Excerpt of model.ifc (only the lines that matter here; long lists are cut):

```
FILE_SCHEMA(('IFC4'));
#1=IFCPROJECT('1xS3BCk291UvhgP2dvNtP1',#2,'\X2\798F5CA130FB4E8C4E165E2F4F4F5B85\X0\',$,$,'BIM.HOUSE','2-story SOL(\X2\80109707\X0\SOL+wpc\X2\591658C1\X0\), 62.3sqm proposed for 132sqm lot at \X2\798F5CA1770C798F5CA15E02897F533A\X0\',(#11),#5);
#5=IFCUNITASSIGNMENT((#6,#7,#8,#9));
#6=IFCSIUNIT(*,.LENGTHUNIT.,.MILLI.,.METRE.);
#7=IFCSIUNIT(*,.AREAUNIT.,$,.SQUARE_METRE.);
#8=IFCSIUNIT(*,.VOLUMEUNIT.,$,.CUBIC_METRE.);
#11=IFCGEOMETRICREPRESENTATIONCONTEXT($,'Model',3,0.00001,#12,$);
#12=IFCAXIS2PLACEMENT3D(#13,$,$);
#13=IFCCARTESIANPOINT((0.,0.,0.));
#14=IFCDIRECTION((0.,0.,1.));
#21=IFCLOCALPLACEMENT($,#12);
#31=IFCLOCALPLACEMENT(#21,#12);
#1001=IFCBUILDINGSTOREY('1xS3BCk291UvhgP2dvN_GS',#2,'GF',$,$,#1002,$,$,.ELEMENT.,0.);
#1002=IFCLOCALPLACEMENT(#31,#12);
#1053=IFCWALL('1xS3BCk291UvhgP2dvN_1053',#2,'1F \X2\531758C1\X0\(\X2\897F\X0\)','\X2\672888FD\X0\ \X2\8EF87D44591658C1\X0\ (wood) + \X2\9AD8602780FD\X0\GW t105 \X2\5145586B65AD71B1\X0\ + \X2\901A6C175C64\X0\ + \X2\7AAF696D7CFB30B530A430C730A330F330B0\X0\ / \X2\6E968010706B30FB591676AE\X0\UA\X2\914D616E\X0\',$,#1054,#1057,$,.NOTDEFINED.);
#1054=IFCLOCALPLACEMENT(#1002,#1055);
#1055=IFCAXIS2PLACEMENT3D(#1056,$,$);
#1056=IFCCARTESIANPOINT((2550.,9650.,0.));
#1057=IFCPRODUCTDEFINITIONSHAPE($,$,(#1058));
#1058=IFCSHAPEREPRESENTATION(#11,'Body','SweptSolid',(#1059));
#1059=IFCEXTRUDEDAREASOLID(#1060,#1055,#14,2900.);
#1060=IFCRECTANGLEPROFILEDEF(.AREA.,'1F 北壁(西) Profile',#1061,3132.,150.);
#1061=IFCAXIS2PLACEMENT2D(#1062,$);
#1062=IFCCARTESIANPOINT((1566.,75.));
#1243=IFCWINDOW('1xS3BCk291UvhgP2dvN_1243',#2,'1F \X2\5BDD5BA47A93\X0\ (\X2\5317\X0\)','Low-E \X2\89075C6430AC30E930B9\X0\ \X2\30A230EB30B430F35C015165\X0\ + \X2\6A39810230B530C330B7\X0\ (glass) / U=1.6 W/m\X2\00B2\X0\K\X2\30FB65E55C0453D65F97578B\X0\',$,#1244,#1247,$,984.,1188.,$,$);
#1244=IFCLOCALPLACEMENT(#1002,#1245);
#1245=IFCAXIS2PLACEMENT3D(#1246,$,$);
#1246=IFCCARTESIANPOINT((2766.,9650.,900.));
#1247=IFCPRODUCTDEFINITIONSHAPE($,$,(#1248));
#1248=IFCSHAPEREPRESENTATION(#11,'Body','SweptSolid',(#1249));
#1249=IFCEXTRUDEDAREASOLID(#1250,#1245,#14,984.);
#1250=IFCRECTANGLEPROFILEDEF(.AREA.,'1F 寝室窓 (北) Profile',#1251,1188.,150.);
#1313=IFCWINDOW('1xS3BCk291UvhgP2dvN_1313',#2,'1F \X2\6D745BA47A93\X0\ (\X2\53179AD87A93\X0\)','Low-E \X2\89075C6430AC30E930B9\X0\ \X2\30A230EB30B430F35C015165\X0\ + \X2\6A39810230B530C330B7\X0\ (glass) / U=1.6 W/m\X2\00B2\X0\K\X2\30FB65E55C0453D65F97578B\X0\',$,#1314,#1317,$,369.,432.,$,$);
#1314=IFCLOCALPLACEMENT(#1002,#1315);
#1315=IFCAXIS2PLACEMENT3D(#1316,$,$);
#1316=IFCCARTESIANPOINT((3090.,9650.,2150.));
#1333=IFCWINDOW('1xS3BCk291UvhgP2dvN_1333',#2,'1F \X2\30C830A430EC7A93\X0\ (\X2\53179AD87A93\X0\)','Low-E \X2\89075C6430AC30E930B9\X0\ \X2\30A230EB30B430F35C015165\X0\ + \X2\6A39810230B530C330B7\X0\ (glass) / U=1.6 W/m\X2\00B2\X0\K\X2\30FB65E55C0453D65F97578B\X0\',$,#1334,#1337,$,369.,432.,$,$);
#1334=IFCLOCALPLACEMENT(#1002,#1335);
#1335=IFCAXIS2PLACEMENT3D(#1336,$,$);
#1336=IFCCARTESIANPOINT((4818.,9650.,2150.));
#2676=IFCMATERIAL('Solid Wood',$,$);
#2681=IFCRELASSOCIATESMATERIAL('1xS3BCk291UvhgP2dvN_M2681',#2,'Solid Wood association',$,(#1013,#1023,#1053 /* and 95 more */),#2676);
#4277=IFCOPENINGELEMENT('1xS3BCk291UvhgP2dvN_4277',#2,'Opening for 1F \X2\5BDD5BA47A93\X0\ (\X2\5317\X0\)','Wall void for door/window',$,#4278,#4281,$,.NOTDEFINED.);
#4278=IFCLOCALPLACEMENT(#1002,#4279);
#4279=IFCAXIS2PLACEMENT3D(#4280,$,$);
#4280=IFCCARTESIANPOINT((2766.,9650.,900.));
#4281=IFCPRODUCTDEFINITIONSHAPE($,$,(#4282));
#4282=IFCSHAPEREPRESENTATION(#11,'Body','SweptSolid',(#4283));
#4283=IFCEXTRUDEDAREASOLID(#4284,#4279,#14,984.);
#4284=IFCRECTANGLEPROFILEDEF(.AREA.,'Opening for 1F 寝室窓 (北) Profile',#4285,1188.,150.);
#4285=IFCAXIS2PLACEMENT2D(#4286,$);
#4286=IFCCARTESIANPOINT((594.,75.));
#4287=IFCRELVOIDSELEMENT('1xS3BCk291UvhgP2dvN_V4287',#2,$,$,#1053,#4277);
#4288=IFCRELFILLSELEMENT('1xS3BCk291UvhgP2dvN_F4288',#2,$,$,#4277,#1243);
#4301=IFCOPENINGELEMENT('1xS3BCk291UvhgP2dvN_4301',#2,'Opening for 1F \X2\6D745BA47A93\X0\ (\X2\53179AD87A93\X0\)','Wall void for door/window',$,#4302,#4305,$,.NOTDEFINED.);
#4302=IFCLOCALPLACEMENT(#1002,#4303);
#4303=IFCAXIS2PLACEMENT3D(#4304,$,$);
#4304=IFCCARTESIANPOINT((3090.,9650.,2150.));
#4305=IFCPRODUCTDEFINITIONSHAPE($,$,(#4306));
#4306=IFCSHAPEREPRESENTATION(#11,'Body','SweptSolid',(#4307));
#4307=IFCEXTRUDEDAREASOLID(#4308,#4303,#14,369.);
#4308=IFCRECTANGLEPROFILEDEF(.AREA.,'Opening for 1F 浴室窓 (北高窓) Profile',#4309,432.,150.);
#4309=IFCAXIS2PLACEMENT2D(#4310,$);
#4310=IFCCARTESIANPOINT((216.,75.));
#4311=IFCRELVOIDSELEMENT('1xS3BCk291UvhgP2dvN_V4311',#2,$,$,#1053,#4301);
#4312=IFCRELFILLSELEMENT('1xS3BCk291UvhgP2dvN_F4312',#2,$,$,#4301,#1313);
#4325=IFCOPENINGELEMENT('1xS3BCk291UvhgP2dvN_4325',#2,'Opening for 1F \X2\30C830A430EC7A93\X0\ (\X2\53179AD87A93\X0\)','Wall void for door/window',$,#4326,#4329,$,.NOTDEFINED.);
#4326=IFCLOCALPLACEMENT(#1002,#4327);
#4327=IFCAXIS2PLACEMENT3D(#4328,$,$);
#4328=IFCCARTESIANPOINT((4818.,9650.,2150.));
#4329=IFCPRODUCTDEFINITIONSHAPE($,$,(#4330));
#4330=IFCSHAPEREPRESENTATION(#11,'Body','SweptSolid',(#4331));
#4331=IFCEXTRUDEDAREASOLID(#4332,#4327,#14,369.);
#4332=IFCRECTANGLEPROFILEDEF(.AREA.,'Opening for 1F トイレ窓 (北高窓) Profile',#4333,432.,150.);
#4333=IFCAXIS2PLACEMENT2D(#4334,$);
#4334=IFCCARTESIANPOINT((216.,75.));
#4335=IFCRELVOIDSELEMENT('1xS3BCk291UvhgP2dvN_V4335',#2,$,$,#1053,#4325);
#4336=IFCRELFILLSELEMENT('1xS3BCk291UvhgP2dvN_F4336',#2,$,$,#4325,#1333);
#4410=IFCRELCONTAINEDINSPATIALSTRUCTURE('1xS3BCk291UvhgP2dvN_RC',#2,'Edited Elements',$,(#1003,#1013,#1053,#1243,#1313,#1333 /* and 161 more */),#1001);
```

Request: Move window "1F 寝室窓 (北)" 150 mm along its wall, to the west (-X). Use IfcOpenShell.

```python
import ifcopenshell
import ifcopenshell.api.geometry
import ifcopenshell.util.placement

model = ifcopenshell.open("model.ifc")

window = model.by_guid("1xS3BCk291UvhgP2dvN_1243")
opening = window.FillsVoids[0].RelatingOpeningElement
wall = opening.VoidsElements[0].RelatingBuildingElement

wall_matrix = ifcopenshell.util.placement.get_local_placement(wall.ObjectPlacement)
shift = wall_matrix[:3, 0] * -150.0
before = ifcopenshell.util.placement.get_local_placement(window.ObjectPlacement)[:3, 3].copy()

# The window is not placed relative to its opening, so move both.
for product in (opening, window):
    matrix = ifcopenshell.util.placement.get_local_placement(product.ObjectPlacement)
    matrix[:3, 3] += shift
    ifcopenshell.api.geometry.edit_object_placement(model, product=product, matrix=matrix, is_si=False)

after = ifcopenshell.util.placement.get_local_placement(window.ObjectPlacement)[:3, 3]
print("window moved by", (after - before).round(3) + 0.0)

model.write("model-out.ifc")
```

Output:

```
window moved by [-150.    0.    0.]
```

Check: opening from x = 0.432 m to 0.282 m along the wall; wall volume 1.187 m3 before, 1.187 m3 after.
